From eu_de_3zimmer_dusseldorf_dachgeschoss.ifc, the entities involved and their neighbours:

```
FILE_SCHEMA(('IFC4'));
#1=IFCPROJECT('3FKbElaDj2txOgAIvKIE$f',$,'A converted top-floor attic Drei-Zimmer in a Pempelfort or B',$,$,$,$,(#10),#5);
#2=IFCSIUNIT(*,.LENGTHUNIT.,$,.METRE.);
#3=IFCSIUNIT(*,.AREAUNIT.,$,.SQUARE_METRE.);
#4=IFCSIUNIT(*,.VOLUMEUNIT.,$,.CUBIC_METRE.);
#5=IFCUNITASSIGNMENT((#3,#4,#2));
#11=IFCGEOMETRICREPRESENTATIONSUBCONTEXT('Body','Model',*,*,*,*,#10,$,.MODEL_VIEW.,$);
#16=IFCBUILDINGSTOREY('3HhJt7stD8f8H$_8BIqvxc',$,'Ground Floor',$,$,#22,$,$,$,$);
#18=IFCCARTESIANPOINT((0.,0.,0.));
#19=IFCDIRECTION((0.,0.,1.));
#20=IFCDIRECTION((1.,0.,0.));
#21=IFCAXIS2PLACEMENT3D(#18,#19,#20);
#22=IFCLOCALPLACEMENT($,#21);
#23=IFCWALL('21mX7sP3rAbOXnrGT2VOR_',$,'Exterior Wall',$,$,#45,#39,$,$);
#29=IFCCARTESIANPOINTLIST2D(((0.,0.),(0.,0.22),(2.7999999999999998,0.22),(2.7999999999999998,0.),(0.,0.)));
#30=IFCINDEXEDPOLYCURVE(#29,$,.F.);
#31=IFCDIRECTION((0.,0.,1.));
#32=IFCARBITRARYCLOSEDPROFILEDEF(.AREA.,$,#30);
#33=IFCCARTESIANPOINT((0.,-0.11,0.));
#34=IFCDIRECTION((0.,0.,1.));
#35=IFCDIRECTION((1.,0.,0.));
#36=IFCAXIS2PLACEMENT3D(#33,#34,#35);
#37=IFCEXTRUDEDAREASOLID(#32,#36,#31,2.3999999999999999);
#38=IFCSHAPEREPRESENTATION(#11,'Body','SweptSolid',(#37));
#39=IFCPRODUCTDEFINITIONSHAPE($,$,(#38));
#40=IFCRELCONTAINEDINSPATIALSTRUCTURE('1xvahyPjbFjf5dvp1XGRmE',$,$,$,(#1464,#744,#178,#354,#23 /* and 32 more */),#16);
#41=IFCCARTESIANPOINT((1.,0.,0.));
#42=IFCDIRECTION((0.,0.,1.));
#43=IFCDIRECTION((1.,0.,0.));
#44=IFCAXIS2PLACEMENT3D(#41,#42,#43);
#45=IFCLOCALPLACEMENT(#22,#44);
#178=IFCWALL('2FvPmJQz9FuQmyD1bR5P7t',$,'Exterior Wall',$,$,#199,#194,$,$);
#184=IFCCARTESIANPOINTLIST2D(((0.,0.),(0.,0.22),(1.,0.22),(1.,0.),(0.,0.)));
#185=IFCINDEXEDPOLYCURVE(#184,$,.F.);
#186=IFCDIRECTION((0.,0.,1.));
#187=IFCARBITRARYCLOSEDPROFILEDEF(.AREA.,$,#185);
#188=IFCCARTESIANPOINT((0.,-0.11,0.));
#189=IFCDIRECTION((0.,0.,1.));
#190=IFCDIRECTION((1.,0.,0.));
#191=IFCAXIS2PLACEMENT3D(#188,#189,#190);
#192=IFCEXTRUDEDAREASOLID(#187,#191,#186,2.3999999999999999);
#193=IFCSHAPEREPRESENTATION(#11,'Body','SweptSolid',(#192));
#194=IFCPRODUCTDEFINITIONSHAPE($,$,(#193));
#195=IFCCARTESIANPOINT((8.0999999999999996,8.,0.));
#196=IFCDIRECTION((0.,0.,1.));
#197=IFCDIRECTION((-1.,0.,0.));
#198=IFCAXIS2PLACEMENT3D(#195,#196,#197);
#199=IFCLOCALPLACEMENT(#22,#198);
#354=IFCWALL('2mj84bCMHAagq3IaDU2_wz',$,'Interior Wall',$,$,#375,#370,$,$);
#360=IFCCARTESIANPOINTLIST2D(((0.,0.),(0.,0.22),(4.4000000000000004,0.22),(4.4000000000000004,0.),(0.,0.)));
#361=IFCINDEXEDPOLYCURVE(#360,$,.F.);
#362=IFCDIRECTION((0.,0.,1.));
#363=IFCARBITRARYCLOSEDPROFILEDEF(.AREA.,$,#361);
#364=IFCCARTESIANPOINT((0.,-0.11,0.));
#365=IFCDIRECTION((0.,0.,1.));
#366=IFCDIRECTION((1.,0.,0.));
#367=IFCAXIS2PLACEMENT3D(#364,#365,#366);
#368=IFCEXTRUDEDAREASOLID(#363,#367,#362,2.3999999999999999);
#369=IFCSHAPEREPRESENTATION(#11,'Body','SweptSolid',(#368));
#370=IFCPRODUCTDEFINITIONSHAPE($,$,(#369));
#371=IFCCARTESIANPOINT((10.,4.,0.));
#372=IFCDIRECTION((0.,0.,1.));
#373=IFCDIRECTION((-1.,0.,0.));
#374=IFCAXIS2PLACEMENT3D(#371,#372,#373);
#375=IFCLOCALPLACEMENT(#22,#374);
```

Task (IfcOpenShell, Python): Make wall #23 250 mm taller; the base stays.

```python
import ifcopenshell
import ifcopenshell.geom
import ifcopenshell.util.representation
import ifcopenshell.util.shape
import ifcopenshell.util.unit

model = ifcopenshell.open("eu_de_3zimmer_dusseldorf_dachgeschoss.ifc")
unit_scale = ifcopenshell.util.unit.calculate_unit_scale(model)
settings = ifcopenshell.geom.settings()


def volume(element):
    """Net volume in cubic metres, openings subtracted."""
    shape = ifcopenshell.geom.create_shape(settings, element)
    return ifcopenshell.util.shape.get_volume(shape.geometry)


wall = model.by_guid("21mX7sP3rAbOXnrGT2VOR_")
before = volume(wall)

body = ifcopenshell.util.representation.get_representation(wall, "Model", "Body")
solid = body.Items[0]
old_height = solid.Depth
solid.Depth += 0.25 / unit_scale
after = volume(wall)

print(f"height {old_height:g} -> {solid.Depth:g}, volume {before:.3f} -> {after:.3f} m3")

model.write("eu_de_3zimmer_dusseldorf_dachgeschoss_v2.ifc")
```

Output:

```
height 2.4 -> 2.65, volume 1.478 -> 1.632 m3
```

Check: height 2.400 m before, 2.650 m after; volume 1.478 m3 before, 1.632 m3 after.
